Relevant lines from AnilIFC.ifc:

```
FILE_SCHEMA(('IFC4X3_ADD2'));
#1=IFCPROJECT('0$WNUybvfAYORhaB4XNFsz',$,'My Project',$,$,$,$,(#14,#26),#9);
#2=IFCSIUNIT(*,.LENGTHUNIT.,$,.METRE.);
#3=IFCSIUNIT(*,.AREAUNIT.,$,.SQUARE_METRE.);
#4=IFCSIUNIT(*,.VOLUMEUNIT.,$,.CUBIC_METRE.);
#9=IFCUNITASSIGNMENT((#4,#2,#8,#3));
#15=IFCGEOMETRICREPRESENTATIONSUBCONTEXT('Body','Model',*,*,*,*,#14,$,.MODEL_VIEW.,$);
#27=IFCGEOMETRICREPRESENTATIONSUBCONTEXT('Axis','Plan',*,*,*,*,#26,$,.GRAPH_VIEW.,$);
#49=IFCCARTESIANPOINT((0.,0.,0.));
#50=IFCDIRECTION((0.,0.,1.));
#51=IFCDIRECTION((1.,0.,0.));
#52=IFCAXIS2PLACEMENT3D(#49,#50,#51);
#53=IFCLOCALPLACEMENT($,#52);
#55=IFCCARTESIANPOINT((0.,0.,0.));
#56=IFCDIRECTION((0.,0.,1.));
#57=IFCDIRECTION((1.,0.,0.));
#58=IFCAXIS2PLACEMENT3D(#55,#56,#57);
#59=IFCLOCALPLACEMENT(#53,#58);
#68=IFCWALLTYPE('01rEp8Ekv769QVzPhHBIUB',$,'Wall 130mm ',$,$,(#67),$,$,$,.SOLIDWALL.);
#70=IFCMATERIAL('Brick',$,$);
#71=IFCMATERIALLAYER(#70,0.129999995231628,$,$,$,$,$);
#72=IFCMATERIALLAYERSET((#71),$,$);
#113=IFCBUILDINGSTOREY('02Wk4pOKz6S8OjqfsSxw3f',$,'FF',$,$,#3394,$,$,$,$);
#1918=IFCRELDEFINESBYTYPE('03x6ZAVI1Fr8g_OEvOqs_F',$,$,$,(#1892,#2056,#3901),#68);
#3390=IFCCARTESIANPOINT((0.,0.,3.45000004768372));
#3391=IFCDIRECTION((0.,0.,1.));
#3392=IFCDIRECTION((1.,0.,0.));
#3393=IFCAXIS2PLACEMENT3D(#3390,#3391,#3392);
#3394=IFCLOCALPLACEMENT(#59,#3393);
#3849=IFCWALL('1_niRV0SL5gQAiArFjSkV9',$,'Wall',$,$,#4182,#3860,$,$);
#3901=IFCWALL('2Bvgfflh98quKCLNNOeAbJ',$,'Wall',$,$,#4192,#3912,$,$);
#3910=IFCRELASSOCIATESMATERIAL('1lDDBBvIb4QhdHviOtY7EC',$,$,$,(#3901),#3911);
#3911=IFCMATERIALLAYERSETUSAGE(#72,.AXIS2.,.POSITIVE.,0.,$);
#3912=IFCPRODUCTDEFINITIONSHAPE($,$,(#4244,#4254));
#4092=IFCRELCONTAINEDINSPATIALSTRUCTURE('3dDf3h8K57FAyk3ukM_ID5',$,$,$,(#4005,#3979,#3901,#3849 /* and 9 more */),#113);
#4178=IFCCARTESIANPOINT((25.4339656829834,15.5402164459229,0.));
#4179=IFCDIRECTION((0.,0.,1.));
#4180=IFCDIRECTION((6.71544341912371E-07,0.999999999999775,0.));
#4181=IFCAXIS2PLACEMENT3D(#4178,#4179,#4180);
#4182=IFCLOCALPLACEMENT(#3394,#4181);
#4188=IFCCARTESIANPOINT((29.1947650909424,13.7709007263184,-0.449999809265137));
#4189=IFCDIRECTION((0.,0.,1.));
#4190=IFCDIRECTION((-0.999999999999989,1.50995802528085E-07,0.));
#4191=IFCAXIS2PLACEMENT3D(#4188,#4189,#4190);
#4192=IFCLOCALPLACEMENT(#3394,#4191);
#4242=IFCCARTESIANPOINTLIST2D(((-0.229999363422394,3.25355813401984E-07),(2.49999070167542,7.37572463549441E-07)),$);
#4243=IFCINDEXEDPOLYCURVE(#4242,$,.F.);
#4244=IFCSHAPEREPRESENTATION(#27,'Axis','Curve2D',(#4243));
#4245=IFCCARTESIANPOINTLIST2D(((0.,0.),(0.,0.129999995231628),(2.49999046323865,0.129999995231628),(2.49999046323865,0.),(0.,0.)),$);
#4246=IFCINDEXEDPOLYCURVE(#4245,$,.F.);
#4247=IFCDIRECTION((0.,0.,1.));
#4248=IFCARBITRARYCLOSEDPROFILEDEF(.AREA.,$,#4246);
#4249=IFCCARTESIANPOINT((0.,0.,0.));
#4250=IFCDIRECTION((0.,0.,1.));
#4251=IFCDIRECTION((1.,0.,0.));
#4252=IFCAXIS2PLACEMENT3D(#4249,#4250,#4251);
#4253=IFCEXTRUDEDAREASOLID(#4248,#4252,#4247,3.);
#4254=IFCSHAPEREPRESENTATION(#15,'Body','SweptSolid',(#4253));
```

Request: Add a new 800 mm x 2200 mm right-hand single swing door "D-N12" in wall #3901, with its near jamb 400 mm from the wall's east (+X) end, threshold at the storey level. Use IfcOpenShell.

```python
import numpy as np
import ifcopenshell
import ifcopenshell.api.feature
import ifcopenshell.api.geometry
import ifcopenshell.api.root
import ifcopenshell.api.spatial
import ifcopenshell.geom
import ifcopenshell.util.element
import ifcopenshell.util.placement
import ifcopenshell.util.representation
import ifcopenshell.util.shape
import ifcopenshell.util.unit

model = ifcopenshell.open("AnilIFC.ifc")
unit_scale = ifcopenshell.util.unit.calculate_unit_scale(model)
settings = ifcopenshell.geom.settings()


def volume(element):
    """Net volume in cubic metres, openings subtracted."""
    shape = ifcopenshell.geom.create_shape(settings, element)
    return ifcopenshell.util.shape.get_volume(shape.geometry)


wall = model.by_guid("2Bvgfflh98quKCLNNOeAbJ")
storey = ifcopenshell.util.element.get_container(wall, ifc_class="IfcBuildingStorey")
context = ifcopenshell.util.representation.get_context(model, "Model", "Body", "MODEL_VIEW")
before = volume(wall)

width, height, from_end, sill = 0.8, 2.2, 0.4, 0.0  # metres

# The wall runs along its own X axis, and the end named is its -X end.
wall_shape = ifcopenshell.geom.create_shape(settings, wall)
x, y, z = ifcopenshell.util.shape.get_vertices(wall_shape.geometry).T
start = x.min() + from_end
face, thickness = float(y.min()), float(y.max() - y.min())
wall_matrix = ifcopenshell.util.placement.get_local_placement(wall.ObjectPlacement)
level = ifcopenshell.util.placement.get_local_placement(storey.ObjectPlacement)[2, 3]


def in_wall(x, y):
    """Placement at x, y metres in the wall's axes, at sill height."""
    matrix = wall_matrix.copy()
    matrix[:, 3] = wall_matrix @ np.array([x / unit_scale, y / unit_scale, 0.0, 1.0])
    matrix[2, 3] = level + sill / unit_scale
    return matrix


# Opening: a box that overshoots both wall faces by 50 mm.
opening = ifcopenshell.api.root.create_entity(model, ifc_class="IfcOpeningElement", predefined_type="OPENING")
box = ifcopenshell.api.geometry.add_wall_representation(
    model, context=context, length=width, height=height, thickness=thickness + 0.1
)
ifcopenshell.api.geometry.assign_representation(model, product=opening, representation=box)
ifcopenshell.api.geometry.edit_object_placement(model, product=opening, matrix=in_wall(start, face - 0.05), is_si=False)
ifcopenshell.api.feature.add_feature(model, feature=opening, element=wall)

door = ifcopenshell.api.root.create_entity(model, ifc_class="IfcDoor", name="D-N12", predefined_type="DOOR")
door.OverallWidth, door.OverallHeight = width / unit_scale, height / unit_scale
door.OperationType = "SINGLE_SWING_RIGHT"
body = ifcopenshell.api.geometry.add_door_representation(
    model,
    context=context,
    overall_width=door.OverallWidth,
    overall_height=door.OverallHeight,
    operation_type="SINGLE_SWING_RIGHT",
    lining_properties={"LiningDepth": thickness / unit_scale, "ThresholdDepth": thickness / unit_scale},
)
ifcopenshell.api.geometry.assign_representation(model, product=door, representation=body)
ifcopenshell.api.spatial.assign_container(model, products=[door], relating_structure=storey)
ifcopenshell.api.feature.add_filling(model, opening=opening, element=door)

# The lining spans the wall, so the door starts at the wall face.
ifcopenshell.api.geometry.edit_object_placement(model, product=door, matrix=in_wall(start, face), is_si=False)

after = volume(wall)

print(f"wall volume {before:.3f} -> {after:.3f} m3")

model.write("AnilIFC_v2.ifc")
```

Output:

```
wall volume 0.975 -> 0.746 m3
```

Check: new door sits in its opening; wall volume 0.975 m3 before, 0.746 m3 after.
